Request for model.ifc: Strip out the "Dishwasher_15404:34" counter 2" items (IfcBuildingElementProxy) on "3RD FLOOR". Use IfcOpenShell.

First a look at what the model holds.

```python
import ifcopenshell
import ifcopenshell.util.element

model = ifcopenshell.open("model.ifc")
print(model.schema)
storey = next(s for s in model.by_type("IfcBuildingStorey") if s.Name == "3RD FLOOR")
proxies = [e for e in ifcopenshell.util.element.get_decomposition(storey) if e.is_a("IfcBuildingElementProxy")]
seen = {}
for e in proxies:
    element_type = ifcopenshell.util.element.get_type(e)
    name = element_type.Name if element_type not in (None, e) else None
    seen[name] = seen.get(name, 0) + 1
for name, count in sorted(seen.items(), key=str):
    print(count, "x", name)
```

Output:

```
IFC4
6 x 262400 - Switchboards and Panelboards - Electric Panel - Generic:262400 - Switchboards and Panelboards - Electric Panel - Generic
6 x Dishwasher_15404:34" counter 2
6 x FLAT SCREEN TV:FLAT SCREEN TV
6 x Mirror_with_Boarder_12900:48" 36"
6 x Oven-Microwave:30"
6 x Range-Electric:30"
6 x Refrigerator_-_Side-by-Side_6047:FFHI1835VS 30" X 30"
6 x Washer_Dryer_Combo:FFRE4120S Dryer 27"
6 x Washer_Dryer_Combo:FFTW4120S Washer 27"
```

```python
import ifcopenshell
import ifcopenshell.api.root
import ifcopenshell.util.element

model = ifcopenshell.open("model.ifc")

storey = next(s for s in model.by_type("IfcBuildingStorey") if s.Name == "3RD FLOOR")
proxies = [e for e in ifcopenshell.util.element.get_decomposition(storey) if e.is_a("IfcBuildingElementProxy")]
targets = [e for e in proxies if (t := ifcopenshell.util.element.get_type(e)) not in (None, e) and t.Name == 'Dishwasher_15404:34" counter 2']

for e in targets:
    ifcopenshell.api.root.remove_product(model, product=e)
print(len(targets), "removed")

model.write("model_rev.ifc")
```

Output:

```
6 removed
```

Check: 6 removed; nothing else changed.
